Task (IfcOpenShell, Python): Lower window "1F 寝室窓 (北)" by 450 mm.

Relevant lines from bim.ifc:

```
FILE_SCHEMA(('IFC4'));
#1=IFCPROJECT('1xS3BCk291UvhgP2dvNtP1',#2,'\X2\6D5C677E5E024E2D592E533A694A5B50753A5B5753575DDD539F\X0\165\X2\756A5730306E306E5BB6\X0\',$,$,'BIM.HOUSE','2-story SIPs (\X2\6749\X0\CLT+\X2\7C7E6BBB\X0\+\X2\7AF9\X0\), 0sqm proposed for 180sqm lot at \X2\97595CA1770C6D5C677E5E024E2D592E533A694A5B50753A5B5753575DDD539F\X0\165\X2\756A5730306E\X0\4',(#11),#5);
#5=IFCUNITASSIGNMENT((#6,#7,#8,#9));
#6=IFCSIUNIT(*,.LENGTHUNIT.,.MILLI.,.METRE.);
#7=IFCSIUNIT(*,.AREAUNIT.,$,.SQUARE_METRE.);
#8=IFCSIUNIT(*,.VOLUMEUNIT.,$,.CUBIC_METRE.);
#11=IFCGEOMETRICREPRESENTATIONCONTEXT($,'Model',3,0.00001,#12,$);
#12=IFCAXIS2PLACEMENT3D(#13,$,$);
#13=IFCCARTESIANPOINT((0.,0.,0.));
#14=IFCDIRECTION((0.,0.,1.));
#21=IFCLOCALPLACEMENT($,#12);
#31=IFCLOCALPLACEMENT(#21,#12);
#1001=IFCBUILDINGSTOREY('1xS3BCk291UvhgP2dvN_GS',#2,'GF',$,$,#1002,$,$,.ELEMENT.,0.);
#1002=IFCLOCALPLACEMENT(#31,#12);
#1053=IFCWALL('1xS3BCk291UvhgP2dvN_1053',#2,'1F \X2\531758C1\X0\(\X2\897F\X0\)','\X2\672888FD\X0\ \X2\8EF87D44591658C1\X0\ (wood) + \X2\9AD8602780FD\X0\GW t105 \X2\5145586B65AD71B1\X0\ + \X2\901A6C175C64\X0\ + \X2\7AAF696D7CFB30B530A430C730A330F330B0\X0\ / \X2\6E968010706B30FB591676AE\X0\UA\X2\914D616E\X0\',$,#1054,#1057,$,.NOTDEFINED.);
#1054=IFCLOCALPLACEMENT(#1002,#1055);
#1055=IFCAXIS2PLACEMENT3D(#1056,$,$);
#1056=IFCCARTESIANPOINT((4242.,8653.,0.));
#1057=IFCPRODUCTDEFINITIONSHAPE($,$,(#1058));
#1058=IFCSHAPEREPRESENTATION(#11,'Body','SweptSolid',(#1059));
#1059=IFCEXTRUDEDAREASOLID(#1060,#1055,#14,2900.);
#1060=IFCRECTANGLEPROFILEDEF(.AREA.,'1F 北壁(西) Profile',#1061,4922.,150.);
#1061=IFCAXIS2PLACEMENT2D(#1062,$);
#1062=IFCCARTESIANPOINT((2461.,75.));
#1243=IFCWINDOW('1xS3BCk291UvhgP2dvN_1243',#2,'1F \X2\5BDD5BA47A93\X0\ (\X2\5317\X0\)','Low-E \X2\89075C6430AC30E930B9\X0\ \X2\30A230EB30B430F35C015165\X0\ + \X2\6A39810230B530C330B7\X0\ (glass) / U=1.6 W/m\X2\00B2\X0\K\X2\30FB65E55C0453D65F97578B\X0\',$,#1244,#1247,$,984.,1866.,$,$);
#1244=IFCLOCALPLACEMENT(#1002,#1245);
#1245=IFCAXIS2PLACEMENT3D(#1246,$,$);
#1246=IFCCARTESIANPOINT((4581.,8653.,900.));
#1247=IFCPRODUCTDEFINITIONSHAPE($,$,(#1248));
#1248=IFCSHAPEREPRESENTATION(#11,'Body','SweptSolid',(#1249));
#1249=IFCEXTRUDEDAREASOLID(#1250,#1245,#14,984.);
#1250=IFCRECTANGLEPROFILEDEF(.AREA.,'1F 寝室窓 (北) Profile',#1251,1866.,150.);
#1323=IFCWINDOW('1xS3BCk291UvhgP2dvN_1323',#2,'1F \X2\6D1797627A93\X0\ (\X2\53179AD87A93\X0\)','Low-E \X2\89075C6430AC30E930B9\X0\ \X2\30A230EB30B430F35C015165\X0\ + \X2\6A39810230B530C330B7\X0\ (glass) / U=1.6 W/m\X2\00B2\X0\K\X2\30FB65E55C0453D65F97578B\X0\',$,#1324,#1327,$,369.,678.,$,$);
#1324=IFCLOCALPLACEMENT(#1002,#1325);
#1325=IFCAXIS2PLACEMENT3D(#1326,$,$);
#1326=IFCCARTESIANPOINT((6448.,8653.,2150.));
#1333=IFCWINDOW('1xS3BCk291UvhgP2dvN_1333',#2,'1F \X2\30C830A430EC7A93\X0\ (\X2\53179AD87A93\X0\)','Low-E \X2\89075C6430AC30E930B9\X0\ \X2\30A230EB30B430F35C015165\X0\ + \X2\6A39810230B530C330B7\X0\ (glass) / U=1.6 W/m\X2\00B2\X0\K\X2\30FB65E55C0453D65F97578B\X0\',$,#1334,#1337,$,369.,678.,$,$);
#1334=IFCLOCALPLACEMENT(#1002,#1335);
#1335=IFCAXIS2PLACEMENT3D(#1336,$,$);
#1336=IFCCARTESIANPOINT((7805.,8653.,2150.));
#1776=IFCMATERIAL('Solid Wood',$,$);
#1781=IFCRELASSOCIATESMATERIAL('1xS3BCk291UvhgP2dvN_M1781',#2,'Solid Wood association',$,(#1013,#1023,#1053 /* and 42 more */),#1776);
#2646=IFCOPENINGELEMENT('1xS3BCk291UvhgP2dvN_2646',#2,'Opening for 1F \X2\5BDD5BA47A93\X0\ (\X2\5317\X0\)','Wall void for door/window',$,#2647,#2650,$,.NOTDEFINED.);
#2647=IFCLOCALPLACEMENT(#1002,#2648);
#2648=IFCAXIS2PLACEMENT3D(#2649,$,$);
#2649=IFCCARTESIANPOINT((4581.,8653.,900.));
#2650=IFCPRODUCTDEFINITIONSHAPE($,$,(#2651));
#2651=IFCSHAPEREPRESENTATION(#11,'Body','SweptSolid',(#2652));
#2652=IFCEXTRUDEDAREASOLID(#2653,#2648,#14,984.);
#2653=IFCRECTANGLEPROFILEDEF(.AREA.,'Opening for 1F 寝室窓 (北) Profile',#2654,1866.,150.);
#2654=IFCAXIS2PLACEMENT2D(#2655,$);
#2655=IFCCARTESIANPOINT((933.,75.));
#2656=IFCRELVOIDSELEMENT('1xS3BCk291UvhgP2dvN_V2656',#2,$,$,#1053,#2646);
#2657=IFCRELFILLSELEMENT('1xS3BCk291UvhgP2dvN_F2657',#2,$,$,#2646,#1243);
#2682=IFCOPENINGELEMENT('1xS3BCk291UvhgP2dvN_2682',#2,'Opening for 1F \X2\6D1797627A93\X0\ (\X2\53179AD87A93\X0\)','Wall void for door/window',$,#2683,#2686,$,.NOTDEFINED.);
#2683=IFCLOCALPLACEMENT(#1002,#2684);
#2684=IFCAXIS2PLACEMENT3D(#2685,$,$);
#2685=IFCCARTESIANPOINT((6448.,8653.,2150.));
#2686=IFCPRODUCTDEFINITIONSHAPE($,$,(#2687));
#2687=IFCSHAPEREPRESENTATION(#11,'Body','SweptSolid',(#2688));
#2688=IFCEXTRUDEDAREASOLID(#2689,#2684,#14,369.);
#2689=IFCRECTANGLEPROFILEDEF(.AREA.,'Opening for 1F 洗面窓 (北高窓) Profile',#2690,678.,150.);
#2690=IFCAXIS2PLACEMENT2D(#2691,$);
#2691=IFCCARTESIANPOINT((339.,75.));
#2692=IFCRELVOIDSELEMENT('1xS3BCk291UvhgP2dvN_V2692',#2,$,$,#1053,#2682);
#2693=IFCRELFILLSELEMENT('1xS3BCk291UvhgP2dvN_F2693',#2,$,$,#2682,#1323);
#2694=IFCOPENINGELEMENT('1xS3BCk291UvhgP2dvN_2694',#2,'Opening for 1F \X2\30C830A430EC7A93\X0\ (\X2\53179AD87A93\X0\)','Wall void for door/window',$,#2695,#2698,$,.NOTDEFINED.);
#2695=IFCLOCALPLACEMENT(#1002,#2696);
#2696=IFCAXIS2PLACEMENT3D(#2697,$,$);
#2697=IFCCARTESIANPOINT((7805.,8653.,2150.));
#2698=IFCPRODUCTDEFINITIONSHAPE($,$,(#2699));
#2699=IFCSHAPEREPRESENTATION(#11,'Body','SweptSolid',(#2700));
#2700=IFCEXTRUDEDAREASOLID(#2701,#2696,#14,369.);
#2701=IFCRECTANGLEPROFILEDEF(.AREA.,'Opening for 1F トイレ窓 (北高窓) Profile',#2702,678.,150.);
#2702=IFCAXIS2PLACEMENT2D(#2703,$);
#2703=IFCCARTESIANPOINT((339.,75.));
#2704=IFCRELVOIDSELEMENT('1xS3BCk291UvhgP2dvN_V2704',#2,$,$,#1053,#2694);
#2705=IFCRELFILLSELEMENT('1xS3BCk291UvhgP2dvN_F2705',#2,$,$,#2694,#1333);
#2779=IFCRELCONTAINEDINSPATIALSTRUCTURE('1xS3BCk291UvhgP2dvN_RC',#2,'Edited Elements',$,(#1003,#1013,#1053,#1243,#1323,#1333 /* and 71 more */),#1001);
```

```python
import numpy as np
import ifcopenshell
import ifcopenshell.api.geometry
import ifcopenshell.util.placement
import ifcopenshell.util.unit

model = ifcopenshell.open("bim.ifc")
unit_scale = ifcopenshell.util.unit.calculate_unit_scale(model)

window = model.by_guid("1xS3BCk291UvhgP2dvN_1243")
opening = window.FillsVoids[0].RelatingOpeningElement
dz = -450.0

shift = np.array([0.0, 0.0, dz])
# The window is not placed relative to its opening, so move both.
for product in (opening, window):
    matrix = ifcopenshell.util.placement.get_local_placement(product.ObjectPlacement)
    matrix[:3, 3] += shift
    ifcopenshell.api.geometry.edit_object_placement(model, product=product, matrix=matrix, is_si=False)

print(f"moved by {dz * unit_scale:+.3f} m")

model.write("bim_v2.ifc")
```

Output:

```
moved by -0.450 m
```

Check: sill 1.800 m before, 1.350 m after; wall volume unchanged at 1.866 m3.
